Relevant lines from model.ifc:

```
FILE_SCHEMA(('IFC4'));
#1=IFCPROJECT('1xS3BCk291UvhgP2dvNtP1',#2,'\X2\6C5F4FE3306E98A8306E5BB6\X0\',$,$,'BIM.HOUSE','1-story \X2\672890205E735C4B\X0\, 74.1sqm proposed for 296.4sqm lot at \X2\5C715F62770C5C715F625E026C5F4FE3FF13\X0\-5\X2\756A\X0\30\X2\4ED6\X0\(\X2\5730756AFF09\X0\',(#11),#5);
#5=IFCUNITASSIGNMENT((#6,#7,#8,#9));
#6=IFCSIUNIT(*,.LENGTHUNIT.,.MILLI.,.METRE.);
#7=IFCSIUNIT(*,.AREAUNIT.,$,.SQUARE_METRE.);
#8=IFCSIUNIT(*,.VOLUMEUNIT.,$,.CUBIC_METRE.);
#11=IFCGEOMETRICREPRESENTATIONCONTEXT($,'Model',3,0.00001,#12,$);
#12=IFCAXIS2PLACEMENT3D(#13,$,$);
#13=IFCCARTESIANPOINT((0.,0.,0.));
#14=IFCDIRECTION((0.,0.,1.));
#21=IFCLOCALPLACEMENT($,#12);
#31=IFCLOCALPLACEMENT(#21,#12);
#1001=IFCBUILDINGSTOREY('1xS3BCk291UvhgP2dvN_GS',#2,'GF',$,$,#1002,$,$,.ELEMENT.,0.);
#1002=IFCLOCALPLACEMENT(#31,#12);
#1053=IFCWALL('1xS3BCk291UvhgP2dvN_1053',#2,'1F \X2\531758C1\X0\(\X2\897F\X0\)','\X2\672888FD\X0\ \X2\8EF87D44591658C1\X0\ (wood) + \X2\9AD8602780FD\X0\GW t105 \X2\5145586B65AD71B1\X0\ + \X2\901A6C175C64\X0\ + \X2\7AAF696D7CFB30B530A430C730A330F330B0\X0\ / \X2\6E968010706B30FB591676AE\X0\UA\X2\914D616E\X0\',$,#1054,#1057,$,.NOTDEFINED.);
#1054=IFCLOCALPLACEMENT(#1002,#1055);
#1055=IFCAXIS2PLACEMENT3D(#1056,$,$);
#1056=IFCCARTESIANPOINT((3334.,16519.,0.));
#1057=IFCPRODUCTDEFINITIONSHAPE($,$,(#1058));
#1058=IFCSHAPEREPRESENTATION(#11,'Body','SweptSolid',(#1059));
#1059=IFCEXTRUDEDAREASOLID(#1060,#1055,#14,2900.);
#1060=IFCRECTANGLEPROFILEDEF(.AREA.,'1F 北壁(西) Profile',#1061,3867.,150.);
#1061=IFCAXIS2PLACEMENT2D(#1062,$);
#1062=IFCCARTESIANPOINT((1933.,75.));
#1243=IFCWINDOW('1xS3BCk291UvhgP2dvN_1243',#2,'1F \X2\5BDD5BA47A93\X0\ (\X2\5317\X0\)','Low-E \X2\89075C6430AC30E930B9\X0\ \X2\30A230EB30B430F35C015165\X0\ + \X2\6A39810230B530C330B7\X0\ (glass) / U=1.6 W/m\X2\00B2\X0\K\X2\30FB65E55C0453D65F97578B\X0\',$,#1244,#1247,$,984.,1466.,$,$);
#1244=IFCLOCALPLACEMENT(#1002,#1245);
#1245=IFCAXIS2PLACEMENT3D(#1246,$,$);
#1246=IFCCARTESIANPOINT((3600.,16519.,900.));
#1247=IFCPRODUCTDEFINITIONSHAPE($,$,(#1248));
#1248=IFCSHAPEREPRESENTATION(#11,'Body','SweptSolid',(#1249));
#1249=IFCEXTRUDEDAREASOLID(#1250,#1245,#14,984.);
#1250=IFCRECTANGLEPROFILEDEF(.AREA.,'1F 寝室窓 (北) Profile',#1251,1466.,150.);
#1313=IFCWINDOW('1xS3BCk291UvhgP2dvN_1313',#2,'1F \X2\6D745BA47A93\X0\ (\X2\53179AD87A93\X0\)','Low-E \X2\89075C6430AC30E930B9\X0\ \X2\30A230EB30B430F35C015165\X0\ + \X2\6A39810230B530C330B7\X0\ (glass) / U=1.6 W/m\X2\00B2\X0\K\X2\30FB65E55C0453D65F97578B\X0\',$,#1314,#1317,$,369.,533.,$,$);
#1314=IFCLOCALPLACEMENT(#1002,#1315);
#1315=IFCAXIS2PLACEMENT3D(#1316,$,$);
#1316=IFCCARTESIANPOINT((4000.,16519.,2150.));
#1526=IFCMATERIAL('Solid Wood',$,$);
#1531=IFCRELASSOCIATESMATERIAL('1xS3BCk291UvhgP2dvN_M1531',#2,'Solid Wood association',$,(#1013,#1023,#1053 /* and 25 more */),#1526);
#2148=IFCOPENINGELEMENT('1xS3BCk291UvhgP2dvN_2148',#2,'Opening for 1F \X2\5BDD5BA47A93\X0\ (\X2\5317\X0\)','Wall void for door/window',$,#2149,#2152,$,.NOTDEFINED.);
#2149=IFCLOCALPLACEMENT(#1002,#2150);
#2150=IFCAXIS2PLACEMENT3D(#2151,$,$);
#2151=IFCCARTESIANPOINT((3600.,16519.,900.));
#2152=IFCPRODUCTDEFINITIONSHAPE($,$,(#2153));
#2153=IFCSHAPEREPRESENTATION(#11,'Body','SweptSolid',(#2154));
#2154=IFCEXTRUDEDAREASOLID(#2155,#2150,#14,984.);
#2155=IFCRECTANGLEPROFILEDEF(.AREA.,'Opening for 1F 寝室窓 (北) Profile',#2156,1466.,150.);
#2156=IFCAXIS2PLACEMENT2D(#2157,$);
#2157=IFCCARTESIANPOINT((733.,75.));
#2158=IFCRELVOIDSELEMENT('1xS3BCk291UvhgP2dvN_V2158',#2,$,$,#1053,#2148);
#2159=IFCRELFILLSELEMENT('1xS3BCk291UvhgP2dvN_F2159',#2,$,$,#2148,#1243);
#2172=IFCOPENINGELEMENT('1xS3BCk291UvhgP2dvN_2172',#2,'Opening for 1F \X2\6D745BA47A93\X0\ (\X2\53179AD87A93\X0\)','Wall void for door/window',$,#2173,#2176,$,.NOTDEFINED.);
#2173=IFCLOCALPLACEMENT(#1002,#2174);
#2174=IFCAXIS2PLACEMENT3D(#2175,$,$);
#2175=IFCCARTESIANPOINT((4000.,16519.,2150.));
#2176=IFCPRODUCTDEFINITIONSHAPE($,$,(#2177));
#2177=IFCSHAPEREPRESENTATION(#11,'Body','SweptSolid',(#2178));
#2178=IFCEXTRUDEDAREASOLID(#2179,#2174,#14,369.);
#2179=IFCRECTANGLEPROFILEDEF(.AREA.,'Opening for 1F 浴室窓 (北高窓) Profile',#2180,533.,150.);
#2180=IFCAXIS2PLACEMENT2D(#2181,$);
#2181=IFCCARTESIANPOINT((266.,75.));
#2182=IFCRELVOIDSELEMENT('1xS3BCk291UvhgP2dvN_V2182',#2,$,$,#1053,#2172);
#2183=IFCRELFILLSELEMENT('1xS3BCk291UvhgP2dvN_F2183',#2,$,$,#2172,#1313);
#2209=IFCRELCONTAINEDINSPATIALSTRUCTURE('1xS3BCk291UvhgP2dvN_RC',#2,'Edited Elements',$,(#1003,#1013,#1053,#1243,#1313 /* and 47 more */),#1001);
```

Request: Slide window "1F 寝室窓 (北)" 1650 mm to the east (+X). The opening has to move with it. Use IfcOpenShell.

```python
import ifcopenshell
import ifcopenshell.api.geometry
import ifcopenshell.util.placement

model = ifcopenshell.open("model.ifc")

window = model.by_guid("1xS3BCk291UvhgP2dvN_1243")
opening = window.FillsVoids[0].RelatingOpeningElement
wall = opening.VoidsElements[0].RelatingBuildingElement

wall_matrix = ifcopenshell.util.placement.get_local_placement(wall.ObjectPlacement)
shift = wall_matrix[:3, 0] * 1650.0
before = ifcopenshell.util.placement.get_local_placement(window.ObjectPlacement)[:3, 3].copy()

# The window is not placed relative to its opening, so move both.
for product in (opening, window):
    matrix = ifcopenshell.util.placement.get_local_placement(product.ObjectPlacement)
    matrix[:3, 3] += shift
    ifcopenshell.api.geometry.edit_object_placement(model, product=product, matrix=matrix, is_si=False)

after = ifcopenshell.util.placement.get_local_placement(window.ObjectPlacement)[:3, 3]
print("window moved by", (after - before).round(3) + 0.0)

model.write("model_rev.ifc")
```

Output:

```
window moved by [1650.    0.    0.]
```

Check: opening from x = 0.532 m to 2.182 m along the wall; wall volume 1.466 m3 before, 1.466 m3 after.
